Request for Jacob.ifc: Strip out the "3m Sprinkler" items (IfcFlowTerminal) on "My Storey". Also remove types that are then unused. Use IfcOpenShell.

First a look at what the model holds.

```python
import ifcopenshell
import ifcopenshell.util.element

model = ifcopenshell.open("Jacob.ifc")
print(model.schema)
storey = next(s for s in model.by_type("IfcBuildingStorey") if s.Name == "My Storey")
terminals = [e for e in ifcopenshell.util.element.get_decomposition(storey) if e.is_a("IfcFlowTerminal")]
seen = {}
for e in terminals:
    element_type = ifcopenshell.util.element.get_type(e)
    name = element_type.Name if element_type not in (None, e) else None
    seen[name] = seen.get(name, 0) + 1
for name, count in sorted(seen.items(), key=str):
    print(count, "x", name)
```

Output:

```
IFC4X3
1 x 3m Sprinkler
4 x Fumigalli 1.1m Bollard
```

```python
import ifcopenshell
import ifcopenshell.api.root
import ifcopenshell.util.element

model = ifcopenshell.open("Jacob.ifc")

storey = next(s for s in model.by_type("IfcBuildingStorey") if s.Name == "My Storey")
terminals = [e for e in ifcopenshell.util.element.get_decomposition(storey) if e.is_a("IfcFlowTerminal")]
targets = [e for e in terminals if (t := ifcopenshell.util.element.get_type(e)) not in (None, e) and t.Name == "3m Sprinkler"]
types = {ifcopenshell.util.element.get_type(e) for e in targets} - {None, *targets}

for e in targets:
    ifcopenshell.api.root.remove_product(model, product=e)
print(len(targets), "removed")

unused = [t for t in types if not ifcopenshell.util.element.get_types(t)]
for t in unused:
    ifcopenshell.api.root.remove_product(model, product=t)
print(len(unused), "unused types removed")

model.write("Jacob_v2.ifc")
```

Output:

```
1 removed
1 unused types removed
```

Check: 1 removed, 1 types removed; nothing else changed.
